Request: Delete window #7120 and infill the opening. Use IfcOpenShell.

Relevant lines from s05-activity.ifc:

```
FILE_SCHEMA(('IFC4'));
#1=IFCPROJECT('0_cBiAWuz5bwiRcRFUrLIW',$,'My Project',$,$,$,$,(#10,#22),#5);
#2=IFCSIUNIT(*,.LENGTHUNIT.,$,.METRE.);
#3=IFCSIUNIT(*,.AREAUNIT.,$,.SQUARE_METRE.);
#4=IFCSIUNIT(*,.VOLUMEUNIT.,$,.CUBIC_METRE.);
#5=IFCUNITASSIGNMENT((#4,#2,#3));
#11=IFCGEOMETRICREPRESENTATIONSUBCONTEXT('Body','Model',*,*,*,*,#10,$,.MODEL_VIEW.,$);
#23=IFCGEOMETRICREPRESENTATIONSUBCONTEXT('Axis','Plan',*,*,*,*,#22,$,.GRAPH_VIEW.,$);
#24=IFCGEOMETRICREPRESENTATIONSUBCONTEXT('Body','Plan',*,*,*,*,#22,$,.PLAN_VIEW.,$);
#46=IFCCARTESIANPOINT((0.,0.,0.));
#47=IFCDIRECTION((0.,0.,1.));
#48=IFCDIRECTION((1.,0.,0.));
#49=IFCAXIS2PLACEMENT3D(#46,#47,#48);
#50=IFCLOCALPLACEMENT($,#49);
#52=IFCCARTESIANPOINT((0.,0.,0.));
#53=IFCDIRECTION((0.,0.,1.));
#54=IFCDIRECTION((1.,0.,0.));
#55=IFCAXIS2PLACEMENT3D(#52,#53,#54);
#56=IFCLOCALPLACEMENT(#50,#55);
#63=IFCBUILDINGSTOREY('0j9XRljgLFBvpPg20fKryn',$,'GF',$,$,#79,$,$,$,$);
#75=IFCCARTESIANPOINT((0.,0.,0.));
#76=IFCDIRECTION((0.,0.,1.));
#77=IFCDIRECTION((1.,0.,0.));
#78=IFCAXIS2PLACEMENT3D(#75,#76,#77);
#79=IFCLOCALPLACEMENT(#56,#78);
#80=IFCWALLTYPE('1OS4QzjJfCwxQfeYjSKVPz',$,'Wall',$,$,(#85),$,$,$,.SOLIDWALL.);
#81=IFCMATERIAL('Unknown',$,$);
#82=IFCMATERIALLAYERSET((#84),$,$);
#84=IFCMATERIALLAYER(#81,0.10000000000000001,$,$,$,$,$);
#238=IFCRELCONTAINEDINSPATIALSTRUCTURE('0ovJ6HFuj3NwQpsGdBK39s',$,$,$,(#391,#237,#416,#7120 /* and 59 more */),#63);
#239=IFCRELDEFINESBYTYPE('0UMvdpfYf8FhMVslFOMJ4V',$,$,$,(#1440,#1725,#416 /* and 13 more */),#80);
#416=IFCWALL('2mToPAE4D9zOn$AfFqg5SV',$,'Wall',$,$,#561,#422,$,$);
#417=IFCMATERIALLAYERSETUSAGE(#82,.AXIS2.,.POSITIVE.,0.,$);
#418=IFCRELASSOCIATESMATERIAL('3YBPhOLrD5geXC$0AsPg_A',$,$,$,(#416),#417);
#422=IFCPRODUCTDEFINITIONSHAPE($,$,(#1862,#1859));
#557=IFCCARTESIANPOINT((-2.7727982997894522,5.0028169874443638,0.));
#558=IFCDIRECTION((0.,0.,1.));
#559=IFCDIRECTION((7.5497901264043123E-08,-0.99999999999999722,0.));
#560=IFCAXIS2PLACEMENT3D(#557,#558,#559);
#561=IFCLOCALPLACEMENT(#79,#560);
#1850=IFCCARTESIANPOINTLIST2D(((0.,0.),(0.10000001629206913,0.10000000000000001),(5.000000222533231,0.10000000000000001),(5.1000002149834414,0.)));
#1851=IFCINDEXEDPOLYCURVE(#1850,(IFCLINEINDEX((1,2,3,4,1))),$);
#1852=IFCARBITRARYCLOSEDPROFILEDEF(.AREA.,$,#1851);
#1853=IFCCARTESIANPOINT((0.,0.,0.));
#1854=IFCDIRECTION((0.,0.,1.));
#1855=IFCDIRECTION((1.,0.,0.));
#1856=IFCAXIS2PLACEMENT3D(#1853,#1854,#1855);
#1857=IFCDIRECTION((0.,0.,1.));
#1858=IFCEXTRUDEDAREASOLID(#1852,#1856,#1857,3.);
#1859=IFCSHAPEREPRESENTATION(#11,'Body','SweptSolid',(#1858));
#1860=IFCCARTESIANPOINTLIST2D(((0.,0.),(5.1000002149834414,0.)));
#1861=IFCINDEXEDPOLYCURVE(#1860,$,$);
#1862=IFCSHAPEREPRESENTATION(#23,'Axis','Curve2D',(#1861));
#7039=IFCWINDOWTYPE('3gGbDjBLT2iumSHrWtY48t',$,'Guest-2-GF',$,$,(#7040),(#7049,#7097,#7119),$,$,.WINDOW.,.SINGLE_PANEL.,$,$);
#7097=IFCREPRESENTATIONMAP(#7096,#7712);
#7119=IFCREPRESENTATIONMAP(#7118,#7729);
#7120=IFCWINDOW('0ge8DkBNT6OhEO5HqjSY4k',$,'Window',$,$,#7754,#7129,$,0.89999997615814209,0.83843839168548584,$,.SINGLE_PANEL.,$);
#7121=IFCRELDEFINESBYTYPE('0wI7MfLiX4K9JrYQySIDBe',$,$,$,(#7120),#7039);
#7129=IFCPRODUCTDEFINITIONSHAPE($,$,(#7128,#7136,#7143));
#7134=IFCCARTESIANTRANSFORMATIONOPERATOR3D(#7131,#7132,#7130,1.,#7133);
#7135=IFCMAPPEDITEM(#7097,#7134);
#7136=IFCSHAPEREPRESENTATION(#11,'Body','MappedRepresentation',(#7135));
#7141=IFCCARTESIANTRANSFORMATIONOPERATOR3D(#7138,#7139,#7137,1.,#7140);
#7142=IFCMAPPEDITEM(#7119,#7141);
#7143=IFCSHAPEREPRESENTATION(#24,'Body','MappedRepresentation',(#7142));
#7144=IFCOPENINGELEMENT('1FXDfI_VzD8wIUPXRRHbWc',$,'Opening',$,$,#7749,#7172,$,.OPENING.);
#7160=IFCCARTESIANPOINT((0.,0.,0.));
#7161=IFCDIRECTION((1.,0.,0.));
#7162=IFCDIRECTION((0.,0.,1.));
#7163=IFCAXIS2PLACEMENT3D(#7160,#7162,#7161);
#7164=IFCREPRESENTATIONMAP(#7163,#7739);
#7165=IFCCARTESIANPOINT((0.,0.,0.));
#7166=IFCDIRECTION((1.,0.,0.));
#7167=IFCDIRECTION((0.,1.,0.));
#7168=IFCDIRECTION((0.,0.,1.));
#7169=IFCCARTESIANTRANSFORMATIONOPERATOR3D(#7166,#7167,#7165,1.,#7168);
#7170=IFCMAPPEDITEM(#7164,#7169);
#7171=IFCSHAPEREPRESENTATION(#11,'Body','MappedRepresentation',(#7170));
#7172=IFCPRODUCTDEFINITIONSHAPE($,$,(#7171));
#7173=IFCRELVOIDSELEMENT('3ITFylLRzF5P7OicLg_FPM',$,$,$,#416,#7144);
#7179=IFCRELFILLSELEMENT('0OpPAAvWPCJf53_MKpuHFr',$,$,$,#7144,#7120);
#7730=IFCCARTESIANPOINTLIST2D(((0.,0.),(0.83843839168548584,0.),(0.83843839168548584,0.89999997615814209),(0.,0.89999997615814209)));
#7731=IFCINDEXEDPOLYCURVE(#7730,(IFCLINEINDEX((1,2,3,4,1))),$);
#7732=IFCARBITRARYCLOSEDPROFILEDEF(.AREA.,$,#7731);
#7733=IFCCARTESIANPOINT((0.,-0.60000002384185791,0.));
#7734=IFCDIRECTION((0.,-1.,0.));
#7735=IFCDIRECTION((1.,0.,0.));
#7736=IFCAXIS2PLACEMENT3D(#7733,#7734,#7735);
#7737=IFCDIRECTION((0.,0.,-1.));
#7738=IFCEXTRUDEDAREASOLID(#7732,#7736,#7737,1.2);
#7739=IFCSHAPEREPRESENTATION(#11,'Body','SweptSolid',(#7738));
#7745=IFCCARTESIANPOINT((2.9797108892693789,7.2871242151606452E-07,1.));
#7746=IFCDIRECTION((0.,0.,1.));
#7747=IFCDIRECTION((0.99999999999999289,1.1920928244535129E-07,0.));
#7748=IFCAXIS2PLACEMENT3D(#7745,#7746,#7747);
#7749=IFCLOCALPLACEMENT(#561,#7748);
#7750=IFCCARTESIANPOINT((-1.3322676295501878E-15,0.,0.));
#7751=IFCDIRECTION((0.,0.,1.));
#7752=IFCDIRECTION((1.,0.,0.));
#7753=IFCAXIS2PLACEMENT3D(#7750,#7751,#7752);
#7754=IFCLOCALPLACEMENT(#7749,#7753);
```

```python
import ifcopenshell
import ifcopenshell.api.feature
import ifcopenshell.api.root
import ifcopenshell.geom
import ifcopenshell.util.shape

model = ifcopenshell.open("s05-activity.ifc")
settings = ifcopenshell.geom.settings()


def volume(element):
    """Net volume in cubic metres, openings subtracted."""
    shape = ifcopenshell.geom.create_shape(settings, element)
    return ifcopenshell.util.shape.get_volume(shape.geometry)


window = model.by_guid("0ge8DkBNT6OhEO5HqjSY4k")
opening = window.FillsVoids[0].RelatingOpeningElement
wall = opening.VoidsElements[0].RelatingBuildingElement
before = volume(wall)

ifcopenshell.api.root.remove_product(model, product=window)
ifcopenshell.api.feature.remove_feature(model, feature=opening)

after = volume(wall)

print(f"wall volume {before:.3f} -> {after:.3f} m3")

model.write("s05-activity-out.ifc")
```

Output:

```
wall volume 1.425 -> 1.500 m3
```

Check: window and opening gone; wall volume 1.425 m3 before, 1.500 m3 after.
